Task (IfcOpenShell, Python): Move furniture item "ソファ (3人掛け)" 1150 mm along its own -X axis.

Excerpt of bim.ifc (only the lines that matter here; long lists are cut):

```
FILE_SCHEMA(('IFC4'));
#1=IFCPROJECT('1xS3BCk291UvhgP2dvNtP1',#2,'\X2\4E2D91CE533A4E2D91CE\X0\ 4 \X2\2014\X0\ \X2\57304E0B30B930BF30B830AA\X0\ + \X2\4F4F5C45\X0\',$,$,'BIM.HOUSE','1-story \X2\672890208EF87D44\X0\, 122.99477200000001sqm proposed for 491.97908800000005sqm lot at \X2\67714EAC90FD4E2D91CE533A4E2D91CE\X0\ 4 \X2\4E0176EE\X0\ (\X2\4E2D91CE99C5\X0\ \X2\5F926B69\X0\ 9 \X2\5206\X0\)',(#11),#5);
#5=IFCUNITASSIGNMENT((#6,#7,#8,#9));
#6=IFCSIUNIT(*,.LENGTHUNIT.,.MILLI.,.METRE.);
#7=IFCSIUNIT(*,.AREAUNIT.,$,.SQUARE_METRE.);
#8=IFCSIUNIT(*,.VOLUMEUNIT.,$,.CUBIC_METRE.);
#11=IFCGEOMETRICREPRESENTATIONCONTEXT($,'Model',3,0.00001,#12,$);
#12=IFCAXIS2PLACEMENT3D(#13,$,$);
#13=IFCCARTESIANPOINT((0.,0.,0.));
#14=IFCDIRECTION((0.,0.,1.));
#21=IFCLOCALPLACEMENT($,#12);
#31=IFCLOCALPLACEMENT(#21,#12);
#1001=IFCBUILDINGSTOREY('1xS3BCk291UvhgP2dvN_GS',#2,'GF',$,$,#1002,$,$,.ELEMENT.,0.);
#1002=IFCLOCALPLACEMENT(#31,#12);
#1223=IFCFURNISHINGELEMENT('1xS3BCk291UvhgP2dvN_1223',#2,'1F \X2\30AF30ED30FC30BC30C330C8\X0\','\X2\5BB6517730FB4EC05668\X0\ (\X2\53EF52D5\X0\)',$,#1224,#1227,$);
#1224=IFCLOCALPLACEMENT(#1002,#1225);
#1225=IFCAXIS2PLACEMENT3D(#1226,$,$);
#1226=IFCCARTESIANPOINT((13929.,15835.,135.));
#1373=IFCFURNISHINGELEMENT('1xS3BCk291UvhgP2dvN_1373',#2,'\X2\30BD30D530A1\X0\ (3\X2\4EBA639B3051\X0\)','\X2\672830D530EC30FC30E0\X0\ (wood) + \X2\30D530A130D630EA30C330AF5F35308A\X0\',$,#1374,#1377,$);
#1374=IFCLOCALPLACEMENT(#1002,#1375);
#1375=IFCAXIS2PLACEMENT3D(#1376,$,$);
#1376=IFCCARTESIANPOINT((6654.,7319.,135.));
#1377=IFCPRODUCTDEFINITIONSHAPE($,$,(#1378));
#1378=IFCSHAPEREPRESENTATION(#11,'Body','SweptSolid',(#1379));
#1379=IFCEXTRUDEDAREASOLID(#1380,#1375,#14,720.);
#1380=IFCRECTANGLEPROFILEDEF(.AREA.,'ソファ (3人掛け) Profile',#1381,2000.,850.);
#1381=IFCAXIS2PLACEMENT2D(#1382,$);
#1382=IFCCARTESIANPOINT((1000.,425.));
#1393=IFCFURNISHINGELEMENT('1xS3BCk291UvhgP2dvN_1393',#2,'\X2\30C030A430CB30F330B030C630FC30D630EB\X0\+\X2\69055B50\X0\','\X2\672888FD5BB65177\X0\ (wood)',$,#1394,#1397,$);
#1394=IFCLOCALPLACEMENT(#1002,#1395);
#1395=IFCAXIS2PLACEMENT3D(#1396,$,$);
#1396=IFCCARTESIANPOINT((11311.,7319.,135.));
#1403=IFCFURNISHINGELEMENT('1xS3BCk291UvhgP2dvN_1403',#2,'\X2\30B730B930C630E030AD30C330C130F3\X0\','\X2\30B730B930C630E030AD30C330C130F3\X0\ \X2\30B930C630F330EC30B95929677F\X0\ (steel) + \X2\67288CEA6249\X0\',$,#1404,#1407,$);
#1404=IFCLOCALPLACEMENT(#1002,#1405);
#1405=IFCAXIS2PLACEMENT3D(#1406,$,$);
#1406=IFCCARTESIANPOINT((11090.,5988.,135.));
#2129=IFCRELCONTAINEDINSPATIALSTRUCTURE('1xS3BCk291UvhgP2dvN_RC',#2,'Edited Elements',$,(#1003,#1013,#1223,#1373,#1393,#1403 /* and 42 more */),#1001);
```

```python
import ifcopenshell
import ifcopenshell.api.geometry
import ifcopenshell.util.placement

model = ifcopenshell.open("bim.ifc")

item = model.by_guid("1xS3BCk291UvhgP2dvN_1373")
matrix = ifcopenshell.util.placement.get_local_placement(item.ObjectPlacement)
matrix[:3, 3] -= matrix[:3, 0] * 1150.0
ifcopenshell.api.geometry.edit_object_placement(model, product=item, matrix=matrix, is_si=False)

print(ifcopenshell.util.placement.get_local_placement(item.ObjectPlacement).round(3) + 0.0)

model.write("bim_updated.ifc")
```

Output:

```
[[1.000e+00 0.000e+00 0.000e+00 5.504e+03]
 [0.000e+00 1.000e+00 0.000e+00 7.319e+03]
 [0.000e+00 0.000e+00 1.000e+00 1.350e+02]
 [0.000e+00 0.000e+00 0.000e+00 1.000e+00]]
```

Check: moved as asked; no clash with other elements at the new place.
